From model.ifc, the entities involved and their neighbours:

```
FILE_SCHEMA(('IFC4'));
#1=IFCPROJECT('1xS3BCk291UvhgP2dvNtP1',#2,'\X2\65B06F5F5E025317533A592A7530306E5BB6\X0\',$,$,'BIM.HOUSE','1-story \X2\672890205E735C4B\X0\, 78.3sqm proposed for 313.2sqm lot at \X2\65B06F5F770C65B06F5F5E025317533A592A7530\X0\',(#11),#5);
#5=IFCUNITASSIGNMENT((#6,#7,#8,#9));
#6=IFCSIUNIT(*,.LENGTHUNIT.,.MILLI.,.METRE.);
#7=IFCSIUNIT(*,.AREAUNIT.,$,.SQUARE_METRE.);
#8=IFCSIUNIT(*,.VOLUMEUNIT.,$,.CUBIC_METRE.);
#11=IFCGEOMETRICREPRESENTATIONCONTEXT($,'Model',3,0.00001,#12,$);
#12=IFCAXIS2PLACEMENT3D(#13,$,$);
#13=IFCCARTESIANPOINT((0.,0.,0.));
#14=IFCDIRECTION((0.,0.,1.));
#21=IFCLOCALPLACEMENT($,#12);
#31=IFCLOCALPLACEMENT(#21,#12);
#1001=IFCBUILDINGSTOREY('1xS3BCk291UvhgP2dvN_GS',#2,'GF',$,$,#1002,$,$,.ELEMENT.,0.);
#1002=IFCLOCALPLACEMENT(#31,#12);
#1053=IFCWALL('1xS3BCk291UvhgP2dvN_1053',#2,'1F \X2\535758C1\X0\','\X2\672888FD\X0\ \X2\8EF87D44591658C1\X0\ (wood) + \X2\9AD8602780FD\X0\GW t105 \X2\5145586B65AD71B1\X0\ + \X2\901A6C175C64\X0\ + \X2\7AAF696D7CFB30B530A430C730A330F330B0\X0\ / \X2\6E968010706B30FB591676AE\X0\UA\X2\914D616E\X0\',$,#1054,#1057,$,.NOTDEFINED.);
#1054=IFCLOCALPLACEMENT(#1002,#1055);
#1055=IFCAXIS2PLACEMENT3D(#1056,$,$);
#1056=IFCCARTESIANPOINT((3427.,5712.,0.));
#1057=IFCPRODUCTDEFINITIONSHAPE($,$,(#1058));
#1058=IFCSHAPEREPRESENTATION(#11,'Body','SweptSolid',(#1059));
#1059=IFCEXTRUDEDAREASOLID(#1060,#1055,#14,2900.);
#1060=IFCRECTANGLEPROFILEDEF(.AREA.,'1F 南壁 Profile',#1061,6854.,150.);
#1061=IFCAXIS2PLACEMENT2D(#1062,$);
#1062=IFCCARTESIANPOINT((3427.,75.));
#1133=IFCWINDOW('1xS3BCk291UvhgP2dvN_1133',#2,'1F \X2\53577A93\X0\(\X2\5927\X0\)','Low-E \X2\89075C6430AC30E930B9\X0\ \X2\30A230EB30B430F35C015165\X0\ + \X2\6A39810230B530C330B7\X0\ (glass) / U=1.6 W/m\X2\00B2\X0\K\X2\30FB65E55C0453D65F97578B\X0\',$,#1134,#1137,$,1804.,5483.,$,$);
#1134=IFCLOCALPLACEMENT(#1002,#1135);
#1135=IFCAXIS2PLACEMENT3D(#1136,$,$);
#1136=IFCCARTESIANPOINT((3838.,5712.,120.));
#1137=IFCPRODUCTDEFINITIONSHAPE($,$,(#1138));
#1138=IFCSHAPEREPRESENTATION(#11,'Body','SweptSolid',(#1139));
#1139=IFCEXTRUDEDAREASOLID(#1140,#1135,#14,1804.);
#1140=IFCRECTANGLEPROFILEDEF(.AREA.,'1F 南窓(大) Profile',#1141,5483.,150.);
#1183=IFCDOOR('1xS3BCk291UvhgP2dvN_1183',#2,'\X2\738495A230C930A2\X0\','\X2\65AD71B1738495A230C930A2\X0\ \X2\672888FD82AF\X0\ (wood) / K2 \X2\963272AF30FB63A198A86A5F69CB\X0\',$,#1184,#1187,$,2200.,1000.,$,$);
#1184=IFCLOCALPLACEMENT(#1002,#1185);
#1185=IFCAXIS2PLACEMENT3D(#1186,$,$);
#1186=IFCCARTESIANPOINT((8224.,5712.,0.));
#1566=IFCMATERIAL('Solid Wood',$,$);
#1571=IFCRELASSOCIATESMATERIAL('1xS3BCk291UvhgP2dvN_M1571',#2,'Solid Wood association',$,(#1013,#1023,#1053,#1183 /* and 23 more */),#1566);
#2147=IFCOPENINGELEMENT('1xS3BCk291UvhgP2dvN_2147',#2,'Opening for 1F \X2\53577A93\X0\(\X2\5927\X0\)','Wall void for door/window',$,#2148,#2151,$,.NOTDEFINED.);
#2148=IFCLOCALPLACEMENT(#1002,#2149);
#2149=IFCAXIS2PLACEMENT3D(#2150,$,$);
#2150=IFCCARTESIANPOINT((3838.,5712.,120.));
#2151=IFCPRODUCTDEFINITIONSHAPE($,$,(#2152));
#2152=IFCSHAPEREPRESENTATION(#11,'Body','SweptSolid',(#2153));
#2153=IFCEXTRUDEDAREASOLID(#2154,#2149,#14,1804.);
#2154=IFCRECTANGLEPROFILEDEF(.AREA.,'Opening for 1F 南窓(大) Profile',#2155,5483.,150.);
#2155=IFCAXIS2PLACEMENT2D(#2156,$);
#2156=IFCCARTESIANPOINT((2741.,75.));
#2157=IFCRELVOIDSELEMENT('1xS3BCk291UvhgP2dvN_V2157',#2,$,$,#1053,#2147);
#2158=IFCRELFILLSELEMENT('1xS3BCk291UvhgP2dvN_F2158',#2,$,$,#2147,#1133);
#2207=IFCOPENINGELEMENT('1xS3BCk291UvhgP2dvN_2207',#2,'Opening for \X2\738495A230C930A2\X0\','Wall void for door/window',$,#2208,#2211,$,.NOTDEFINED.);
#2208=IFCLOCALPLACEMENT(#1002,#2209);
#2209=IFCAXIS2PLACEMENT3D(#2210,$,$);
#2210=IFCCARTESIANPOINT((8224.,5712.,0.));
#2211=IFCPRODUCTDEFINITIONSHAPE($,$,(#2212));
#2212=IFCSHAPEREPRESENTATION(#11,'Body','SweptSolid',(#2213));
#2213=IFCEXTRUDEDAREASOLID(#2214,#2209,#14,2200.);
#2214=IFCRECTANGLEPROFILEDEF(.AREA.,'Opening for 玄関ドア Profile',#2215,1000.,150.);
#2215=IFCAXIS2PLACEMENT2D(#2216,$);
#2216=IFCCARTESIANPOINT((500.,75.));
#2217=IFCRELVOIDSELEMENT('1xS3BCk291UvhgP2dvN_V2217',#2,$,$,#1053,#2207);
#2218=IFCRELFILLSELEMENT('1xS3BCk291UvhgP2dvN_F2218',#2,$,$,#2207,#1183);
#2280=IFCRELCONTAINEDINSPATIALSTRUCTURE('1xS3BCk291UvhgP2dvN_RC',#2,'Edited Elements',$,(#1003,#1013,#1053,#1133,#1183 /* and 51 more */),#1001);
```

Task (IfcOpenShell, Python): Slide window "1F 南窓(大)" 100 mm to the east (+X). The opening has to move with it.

```python
import ifcopenshell
import ifcopenshell.api.geometry
import ifcopenshell.util.placement

model = ifcopenshell.open("model.ifc")

window = model.by_guid("1xS3BCk291UvhgP2dvN_1133")
opening = window.FillsVoids[0].RelatingOpeningElement
wall = opening.VoidsElements[0].RelatingBuildingElement

wall_matrix = ifcopenshell.util.placement.get_local_placement(wall.ObjectPlacement)
shift = wall_matrix[:3, 0] * 100.0
before = ifcopenshell.util.placement.get_local_placement(window.ObjectPlacement)[:3, 3].copy()

# The window is not placed relative to its opening, so move both.
for product in (opening, window):
    matrix = ifcopenshell.util.placement.get_local_placement(product.ObjectPlacement)
    matrix[:3, 3] += shift
    ifcopenshell.api.geometry.edit_object_placement(model, product=product, matrix=matrix, is_si=False)

after = ifcopenshell.util.placement.get_local_placement(window.ObjectPlacement)[:3, 3]
print("window moved by", (after - before).round(3) + 0.0)

model.write("model_updated.ifc")
```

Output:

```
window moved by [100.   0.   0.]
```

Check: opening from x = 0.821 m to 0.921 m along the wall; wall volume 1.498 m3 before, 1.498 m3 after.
